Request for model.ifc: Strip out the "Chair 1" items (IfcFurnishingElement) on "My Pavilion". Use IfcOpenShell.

First a look at what the model holds.

```python
import ifcopenshell
import ifcopenshell.util.element

model = ifcopenshell.open("model.ifc")
print(model.schema)
storey = next(s for s in model.by_type("IfcBuildingStorey") if s.Name == "My Pavilion")
furniture = [e for e in ifcopenshell.util.element.get_decomposition(storey) if e.is_a("IfcFurnishingElement")]
seen = {}
for e in furniture:
    element_type = ifcopenshell.util.element.get_type(e)
    name = element_type.Name if element_type not in (None, e) else None
    seen[name] = seen.get(name, 0) + 1
for name, count in sorted(seen.items(), key=str):
    print(count, "x", name)
```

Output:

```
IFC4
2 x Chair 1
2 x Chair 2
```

```python
import ifcopenshell
import ifcopenshell.api.root
import ifcopenshell.util.element

model = ifcopenshell.open("model.ifc")

storey = next(s for s in model.by_type("IfcBuildingStorey") if s.Name == "My Pavilion")
furniture = [e for e in ifcopenshell.util.element.get_decomposition(storey) if e.is_a("IfcFurnishingElement")]
targets = [e for e in furniture if (t := ifcopenshell.util.element.get_type(e)) not in (None, e) and t.Name == "Chair 1"]

for e in targets:
    ifcopenshell.api.root.remove_product(model, product=e)
print(len(targets), "removed")

model.write("model_updated.ifc")
```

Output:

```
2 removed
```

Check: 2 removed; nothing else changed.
